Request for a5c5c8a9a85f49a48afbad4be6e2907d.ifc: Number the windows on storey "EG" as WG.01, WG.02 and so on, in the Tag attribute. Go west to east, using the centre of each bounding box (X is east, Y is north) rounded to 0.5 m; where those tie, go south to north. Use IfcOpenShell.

First a look at what the model holds.

```python
import ifcopenshell
import ifcopenshell.util.element
import ifcopenshell.util.placement

model = ifcopenshell.open("a5c5c8a9a85f49a48afbad4be6e2907d.ifc")
print(model.schema)
storey = next(s for s in model.by_type("IfcBuildingStorey") if s.Name == "EG")
windows = [e for e in ifcopenshell.util.element.get_decomposition(storey) if e.is_a("IfcWindow")]
for e in sorted(windows, key=lambda e: e.id()):
    origin = ifcopenshell.util.placement.get_local_placement(e.ObjectPlacement)[:3, 3]
    print(e.id(), e.Tag, e.Name, origin.round(2) + 0.0, sep=" | ")
```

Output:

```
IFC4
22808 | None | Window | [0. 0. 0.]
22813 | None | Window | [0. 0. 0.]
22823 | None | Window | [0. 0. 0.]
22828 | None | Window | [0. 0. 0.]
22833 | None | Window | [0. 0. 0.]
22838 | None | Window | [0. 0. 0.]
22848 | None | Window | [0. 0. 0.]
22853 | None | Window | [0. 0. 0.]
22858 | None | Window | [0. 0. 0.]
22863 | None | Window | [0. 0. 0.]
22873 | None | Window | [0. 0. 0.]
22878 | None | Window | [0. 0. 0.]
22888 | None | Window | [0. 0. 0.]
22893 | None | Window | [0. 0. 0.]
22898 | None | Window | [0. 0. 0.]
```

```python
import ifcopenshell
import ifcopenshell.geom
import ifcopenshell.util.element
import ifcopenshell.util.shape

model = ifcopenshell.open("a5c5c8a9a85f49a48afbad4be6e2907d.ifc")
settings = ifcopenshell.geom.settings()
settings.set("use-world-coords", True)


def centre(element):
    shape = ifcopenshell.geom.create_shape(settings, element)
    return ifcopenshell.util.shape.get_bbox_centroid(shape.geometry)


storey = next(s for s in model.by_type("IfcBuildingStorey") if s.Name == "EG")
windows = [e for e in ifcopenshell.util.element.get_decomposition(storey) if e.is_a("IfcWindow")]

# Insertion points can sit at a corner or the storey origin, so sort by the geometry (in metres).
centres = {e: centre(e) for e in windows}
windows.sort(key=lambda e: (round(centres[e][0] / 0.5), centres[e][1]))

for i, e in enumerate(windows, start=1):
    number = f"WG.{i:02d}"
    e.Tag = number
    print(e.id(), number)

model.write("a5c5c8a9a85f49a48afbad4be6e2907d_v2.ifc")
```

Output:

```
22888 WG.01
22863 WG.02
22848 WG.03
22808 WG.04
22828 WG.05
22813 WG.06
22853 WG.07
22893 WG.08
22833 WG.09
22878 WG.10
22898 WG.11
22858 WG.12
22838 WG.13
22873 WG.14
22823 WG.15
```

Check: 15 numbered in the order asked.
